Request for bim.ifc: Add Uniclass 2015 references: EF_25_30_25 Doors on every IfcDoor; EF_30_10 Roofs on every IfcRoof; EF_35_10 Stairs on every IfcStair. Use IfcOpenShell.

First a look at what the model holds.

```python
import ifcopenshell

model = ifcopenshell.open("bim.ifc")
print(model.schema)
print("classifications:", [c.Name for c in model.by_type("IfcClassification")])
for ifc_class in ("IfcDoor", "IfcRoof", "IfcStair", "IfcWall", "IfcWindow"):
    print(ifc_class, len(model.by_type(ifc_class)))
```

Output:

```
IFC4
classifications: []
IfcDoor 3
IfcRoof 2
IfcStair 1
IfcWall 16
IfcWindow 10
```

```python
import ifcopenshell
import ifcopenshell.api.classification

model = ifcopenshell.open("bim.ifc")

system = ifcopenshell.api.classification.add_classification(model, classification="Uniclass 2015")

codes = {
    "IfcDoor": ("EF_25_30_25", "Doors"),
    "IfcRoof": ("EF_30_10", "Roofs"),
    "IfcStair": ("EF_35_10", "Stairs"),
}
for ifc_class, (code, name) in codes.items():
    products = model.by_type(ifc_class)
    ifcopenshell.api.classification.add_reference(
        model, products=products, classification=system, identification=code, name=name
    )
    print(code, len(products))

model.write("bim_rev.ifc")
```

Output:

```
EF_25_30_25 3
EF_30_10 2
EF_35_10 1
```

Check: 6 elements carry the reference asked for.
